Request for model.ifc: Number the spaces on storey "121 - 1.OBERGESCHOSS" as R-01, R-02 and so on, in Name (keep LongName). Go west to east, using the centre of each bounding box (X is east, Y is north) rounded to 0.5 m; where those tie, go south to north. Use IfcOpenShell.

First a look at what the model holds.

```python
import ifcopenshell
import ifcopenshell.util.element
import ifcopenshell.util.placement

model = ifcopenshell.open("model.ifc")
print(model.schema)
storey = next(s for s in model.by_type("IfcBuildingStorey") if s.Name == "121 - 1.OBERGESCHOSS")
spaces = [e for e in ifcopenshell.util.element.get_decomposition(storey) if e.is_a("IfcSpace")]
for e in sorted(spaces, key=lambda e: e.id()):
    origin = ifcopenshell.util.placement.get_local_placement(e.ObjectPlacement)[:3, 3]
    print(e.id(), e.Name, e.LongName, origin.round(2) + 0.0, sep=" | ")
```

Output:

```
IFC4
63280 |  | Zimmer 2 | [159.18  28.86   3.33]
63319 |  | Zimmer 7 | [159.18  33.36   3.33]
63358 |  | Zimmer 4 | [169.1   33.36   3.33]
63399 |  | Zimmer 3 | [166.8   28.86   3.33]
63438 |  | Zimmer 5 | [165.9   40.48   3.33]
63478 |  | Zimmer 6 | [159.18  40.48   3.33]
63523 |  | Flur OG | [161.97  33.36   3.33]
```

```python
import ifcopenshell
import ifcopenshell.geom
import ifcopenshell.util.element
import ifcopenshell.util.shape

model = ifcopenshell.open("model.ifc")
settings = ifcopenshell.geom.settings()
settings.set("use-world-coords", True)


def centre(element):
    shape = ifcopenshell.geom.create_shape(settings, element)
    return ifcopenshell.util.shape.get_bbox_centroid(shape.geometry)


storey = next(s for s in model.by_type("IfcBuildingStorey") if s.Name == "121 - 1.OBERGESCHOSS")
spaces = [e for e in ifcopenshell.util.element.get_decomposition(storey) if e.is_a("IfcSpace")]

# Insertion points can sit at a corner or the storey origin, so sort by the geometry (in metres).
centres = {e: centre(e) for e in spaces}
spaces.sort(key=lambda e: (round(centres[e][0] / 0.5), centres[e][1]))

for i, e in enumerate(spaces, start=1):
    number = f"R-{i:02d}"
    e.Name = number
    print(e.id(), number)

model.write("model_rev.ifc")
```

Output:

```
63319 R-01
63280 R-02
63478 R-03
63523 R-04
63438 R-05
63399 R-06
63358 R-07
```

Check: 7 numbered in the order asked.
